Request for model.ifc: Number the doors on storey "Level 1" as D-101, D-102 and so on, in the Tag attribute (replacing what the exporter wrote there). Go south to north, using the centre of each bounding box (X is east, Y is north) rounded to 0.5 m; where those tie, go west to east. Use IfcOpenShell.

First a look at what the model holds.

```python
import ifcopenshell
import ifcopenshell.util.element
import ifcopenshell.util.placement

model = ifcopenshell.open("model.ifc")
print(model.schema)
storey = next(s for s in model.by_type("IfcBuildingStorey") if s.Name == "Level 1")
doors = [e for e in ifcopenshell.util.element.get_decomposition(storey) if e.is_a("IfcDoor")]
for e in sorted(doors, key=lambda e: e.id()):
    origin = ifcopenshell.util.placement.get_local_placement(e.ObjectPlacement)[:3, 3]
    print(e.id(), e.Tag, e.Name, origin.round(2) + 0.0, sep=" | ")
```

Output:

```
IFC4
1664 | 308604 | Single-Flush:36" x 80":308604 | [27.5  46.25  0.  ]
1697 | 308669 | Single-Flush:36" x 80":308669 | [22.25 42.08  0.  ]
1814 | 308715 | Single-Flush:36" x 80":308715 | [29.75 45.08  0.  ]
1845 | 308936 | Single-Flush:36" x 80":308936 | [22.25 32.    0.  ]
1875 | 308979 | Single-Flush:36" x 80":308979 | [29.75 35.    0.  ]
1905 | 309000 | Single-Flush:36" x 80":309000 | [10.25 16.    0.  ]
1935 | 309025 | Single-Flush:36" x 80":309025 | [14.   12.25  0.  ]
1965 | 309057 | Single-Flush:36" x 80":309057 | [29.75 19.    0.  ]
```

```python
import ifcopenshell
import ifcopenshell.geom
import ifcopenshell.util.element
import ifcopenshell.util.shape

model = ifcopenshell.open("model.ifc")
settings = ifcopenshell.geom.settings()
settings.set("use-world-coords", True)


def centre(element):
    shape = ifcopenshell.geom.create_shape(settings, element)
    return ifcopenshell.util.shape.get_bbox_centroid(shape.geometry)


storey = next(s for s in model.by_type("IfcBuildingStorey") if s.Name == "Level 1")
doors = [e for e in ifcopenshell.util.element.get_decomposition(storey) if e.is_a("IfcDoor")]

# Insertion points can sit at a corner or the storey origin, so sort by the geometry (in metres).
centres = {e: centre(e) for e in doors}
doors.sort(key=lambda e: (round(centres[e][1] / 0.5), centres[e][0]))

for i, e in enumerate(doors, start=1):
    number = f"D-1{i:02d}"
    e.Tag = number
    print(e.id(), number)

model.write("model_v2.ifc")
```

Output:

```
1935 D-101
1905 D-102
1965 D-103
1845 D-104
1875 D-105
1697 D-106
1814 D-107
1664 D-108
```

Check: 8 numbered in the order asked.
